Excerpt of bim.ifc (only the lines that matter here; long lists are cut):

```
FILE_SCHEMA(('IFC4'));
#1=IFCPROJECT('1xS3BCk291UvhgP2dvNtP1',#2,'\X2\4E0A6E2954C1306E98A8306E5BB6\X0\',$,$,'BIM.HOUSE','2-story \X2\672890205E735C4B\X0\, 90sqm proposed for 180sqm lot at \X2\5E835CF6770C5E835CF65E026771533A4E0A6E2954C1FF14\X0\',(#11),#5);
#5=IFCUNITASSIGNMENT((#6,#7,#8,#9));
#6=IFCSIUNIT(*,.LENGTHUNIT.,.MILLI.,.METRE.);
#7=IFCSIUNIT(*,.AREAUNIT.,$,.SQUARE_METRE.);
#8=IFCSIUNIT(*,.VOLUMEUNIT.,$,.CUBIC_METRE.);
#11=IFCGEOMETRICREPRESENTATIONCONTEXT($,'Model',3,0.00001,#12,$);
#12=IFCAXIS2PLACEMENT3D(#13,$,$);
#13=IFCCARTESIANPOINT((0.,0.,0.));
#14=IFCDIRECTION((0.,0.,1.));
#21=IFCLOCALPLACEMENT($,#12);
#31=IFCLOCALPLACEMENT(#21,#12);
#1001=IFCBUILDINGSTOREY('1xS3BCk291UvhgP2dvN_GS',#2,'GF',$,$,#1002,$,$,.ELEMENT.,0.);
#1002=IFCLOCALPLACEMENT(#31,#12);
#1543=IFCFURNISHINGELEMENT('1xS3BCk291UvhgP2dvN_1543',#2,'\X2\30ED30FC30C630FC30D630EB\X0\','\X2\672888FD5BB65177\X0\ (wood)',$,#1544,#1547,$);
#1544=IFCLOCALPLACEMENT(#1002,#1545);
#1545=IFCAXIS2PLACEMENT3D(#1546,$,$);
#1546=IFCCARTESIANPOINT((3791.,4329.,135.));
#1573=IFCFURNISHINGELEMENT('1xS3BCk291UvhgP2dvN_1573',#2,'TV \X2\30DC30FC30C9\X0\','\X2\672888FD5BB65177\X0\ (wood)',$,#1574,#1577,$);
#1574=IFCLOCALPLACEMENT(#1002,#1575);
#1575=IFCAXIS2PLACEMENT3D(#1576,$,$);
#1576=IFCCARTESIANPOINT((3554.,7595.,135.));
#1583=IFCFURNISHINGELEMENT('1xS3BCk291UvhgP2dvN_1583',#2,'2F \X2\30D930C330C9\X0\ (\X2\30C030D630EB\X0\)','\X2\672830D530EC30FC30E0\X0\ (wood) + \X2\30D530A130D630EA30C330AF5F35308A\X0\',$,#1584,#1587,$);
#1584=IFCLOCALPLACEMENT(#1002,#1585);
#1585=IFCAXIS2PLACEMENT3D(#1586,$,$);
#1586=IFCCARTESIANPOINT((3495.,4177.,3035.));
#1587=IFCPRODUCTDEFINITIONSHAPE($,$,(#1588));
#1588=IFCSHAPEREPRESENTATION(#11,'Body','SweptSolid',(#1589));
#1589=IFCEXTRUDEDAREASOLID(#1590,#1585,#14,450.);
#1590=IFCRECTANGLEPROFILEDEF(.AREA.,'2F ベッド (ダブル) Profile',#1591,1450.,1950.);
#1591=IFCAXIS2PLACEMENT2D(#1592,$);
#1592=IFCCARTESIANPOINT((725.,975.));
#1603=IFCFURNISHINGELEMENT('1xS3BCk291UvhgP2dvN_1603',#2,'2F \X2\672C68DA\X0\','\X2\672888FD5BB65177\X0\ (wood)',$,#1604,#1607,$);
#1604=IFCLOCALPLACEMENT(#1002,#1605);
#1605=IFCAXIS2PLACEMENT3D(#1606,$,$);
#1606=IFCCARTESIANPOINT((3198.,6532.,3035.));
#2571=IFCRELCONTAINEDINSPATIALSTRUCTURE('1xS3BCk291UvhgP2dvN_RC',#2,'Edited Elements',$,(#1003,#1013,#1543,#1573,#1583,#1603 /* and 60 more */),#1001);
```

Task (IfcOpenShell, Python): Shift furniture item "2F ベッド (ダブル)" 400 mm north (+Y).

```python
import ifcopenshell
import ifcopenshell.api.geometry
import ifcopenshell.util.placement

model = ifcopenshell.open("bim.ifc")

item = model.by_guid("1xS3BCk291UvhgP2dvN_1583")
matrix = ifcopenshell.util.placement.get_local_placement(item.ObjectPlacement)
matrix[1, 3] += 400.0
ifcopenshell.api.geometry.edit_object_placement(model, product=item, matrix=matrix, is_si=False)

print(ifcopenshell.util.placement.get_local_placement(item.ObjectPlacement).round(3) + 0.0)

model.write("bim_v2.ifc")
```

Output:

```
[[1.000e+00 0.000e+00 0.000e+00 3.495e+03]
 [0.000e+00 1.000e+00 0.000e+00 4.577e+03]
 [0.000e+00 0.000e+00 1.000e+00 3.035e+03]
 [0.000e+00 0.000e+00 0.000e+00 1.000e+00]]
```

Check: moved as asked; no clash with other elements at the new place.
